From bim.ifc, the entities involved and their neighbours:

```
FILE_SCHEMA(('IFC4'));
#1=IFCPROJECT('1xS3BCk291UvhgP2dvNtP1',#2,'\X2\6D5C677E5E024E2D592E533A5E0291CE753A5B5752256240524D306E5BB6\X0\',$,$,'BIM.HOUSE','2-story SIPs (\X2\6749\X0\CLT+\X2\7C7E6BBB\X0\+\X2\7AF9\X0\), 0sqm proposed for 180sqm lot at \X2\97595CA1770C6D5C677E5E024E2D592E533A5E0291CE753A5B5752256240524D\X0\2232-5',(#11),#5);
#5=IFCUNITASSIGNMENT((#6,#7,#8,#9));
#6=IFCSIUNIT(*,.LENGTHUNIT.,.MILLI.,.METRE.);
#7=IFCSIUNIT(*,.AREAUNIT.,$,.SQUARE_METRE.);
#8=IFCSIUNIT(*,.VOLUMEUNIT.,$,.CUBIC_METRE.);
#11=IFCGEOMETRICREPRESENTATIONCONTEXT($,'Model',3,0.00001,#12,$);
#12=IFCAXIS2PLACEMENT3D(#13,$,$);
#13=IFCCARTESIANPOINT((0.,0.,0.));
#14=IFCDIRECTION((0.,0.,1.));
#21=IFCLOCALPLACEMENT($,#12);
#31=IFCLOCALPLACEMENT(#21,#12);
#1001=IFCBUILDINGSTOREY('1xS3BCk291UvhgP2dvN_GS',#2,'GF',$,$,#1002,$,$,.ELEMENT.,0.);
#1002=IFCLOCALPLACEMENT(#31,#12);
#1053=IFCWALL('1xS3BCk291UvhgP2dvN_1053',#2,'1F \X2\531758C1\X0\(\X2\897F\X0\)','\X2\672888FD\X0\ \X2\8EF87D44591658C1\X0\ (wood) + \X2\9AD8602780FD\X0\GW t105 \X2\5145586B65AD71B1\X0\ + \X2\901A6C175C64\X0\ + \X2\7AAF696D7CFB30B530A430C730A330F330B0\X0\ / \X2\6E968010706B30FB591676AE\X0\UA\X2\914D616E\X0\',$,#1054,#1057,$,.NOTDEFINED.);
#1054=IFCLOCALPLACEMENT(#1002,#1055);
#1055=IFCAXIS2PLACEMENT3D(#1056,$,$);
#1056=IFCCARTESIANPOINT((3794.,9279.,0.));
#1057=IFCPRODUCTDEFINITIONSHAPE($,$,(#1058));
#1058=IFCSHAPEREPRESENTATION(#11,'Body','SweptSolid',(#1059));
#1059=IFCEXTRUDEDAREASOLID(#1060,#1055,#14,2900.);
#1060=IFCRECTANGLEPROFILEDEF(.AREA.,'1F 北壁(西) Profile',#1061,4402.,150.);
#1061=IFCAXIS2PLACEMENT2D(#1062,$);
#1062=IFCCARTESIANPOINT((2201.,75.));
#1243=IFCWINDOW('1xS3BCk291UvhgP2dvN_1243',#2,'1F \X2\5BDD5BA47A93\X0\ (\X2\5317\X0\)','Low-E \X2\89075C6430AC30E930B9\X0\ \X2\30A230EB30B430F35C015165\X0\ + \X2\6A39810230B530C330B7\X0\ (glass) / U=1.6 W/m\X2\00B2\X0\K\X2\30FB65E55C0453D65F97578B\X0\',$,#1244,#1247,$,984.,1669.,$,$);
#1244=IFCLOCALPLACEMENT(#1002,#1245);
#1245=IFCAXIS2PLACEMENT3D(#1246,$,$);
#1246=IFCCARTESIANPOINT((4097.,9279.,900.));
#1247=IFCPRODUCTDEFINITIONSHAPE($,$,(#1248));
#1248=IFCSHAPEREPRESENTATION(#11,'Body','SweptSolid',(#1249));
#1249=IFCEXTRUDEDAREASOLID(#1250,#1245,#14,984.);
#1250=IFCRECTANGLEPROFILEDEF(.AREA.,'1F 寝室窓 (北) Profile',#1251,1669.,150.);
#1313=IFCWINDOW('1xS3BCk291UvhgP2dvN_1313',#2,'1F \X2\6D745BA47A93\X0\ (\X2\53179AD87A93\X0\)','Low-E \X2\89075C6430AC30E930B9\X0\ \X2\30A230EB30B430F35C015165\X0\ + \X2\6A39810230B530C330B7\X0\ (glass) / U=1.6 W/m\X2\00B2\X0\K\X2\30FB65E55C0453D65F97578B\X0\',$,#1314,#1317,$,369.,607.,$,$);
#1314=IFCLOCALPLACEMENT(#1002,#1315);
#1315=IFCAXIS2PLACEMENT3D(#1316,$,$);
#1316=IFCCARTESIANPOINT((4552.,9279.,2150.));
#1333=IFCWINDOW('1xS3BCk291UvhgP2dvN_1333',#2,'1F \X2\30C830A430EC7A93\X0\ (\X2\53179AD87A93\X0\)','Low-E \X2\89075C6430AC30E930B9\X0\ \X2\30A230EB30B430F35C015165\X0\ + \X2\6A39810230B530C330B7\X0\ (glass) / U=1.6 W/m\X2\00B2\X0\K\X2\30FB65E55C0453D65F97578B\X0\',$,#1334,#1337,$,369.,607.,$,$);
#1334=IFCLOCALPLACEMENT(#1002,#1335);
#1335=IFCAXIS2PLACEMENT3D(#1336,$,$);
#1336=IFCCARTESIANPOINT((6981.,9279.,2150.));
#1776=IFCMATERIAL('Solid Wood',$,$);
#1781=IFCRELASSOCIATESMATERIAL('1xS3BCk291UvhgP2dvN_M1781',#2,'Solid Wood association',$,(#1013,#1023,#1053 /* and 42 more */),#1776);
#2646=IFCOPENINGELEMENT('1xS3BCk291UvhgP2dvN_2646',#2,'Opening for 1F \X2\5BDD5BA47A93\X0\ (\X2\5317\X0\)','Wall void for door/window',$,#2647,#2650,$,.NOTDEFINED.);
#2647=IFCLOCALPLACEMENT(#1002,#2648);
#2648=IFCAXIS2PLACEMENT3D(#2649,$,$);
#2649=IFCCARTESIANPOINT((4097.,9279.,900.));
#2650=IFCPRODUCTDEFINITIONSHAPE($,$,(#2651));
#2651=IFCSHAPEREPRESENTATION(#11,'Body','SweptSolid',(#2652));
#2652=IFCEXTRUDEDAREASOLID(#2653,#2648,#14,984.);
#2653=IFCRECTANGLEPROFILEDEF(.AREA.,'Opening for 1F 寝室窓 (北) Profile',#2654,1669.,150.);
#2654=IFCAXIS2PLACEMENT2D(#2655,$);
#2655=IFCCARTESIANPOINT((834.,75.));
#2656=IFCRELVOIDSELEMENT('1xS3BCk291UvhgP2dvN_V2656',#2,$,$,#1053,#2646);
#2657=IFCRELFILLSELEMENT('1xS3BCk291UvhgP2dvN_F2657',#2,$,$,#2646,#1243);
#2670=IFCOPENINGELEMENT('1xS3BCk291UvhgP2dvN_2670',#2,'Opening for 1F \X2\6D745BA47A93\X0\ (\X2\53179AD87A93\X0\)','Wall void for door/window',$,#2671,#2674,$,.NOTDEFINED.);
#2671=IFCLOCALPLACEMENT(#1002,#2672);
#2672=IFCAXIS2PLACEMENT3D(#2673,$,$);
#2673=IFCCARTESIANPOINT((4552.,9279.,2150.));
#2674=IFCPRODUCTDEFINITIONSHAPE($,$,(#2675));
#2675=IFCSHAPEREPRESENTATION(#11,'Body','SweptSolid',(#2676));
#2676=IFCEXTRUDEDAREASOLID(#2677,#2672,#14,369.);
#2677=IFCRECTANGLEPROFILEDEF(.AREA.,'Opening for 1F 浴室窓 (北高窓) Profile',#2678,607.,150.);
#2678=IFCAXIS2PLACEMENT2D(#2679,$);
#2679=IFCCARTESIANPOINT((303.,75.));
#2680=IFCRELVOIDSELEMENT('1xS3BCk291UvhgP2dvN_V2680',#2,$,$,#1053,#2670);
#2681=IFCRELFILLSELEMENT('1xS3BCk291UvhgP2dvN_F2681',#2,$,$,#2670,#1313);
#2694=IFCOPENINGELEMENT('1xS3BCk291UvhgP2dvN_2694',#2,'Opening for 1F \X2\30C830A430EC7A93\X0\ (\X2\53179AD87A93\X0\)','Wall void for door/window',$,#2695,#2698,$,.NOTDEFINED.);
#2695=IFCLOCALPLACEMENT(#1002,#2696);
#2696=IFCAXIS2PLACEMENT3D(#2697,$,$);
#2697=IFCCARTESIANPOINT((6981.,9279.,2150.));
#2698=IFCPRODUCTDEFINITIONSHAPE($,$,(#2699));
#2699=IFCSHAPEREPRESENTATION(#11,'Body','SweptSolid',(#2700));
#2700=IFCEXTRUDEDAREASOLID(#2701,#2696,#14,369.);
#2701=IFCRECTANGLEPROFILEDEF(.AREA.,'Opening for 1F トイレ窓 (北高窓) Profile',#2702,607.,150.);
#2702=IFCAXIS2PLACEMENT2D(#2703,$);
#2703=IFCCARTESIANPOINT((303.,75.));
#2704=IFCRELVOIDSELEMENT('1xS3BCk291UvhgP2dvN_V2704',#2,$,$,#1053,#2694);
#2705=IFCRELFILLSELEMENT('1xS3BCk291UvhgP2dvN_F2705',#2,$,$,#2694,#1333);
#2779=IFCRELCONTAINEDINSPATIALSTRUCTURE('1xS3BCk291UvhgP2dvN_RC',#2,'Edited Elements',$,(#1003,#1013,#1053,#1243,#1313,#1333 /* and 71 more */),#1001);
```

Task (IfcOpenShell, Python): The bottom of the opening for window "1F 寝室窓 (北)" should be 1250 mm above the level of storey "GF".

```python
import numpy as np
import ifcopenshell
import ifcopenshell.api.geometry
import ifcopenshell.geom
import ifcopenshell.util.element
import ifcopenshell.util.placement
import ifcopenshell.util.shape
import ifcopenshell.util.unit

model = ifcopenshell.open("bim.ifc")
unit_scale = ifcopenshell.util.unit.calculate_unit_scale(model)

window = model.by_id(1243)
opening = window.FillsVoids[0].RelatingOpeningElement
storey = ifcopenshell.util.element.get_container(window, ifc_class="IfcBuildingStorey")
level = ifcopenshell.util.placement.get_local_placement(storey.ObjectPlacement)[2, 3]

# The opening's origin need not be at the sill, so measure its lowest point.
shape = ifcopenshell.geom.create_shape(ifcopenshell.geom.settings(), opening)
bottom = ifcopenshell.util.shape.get_shape_bottom_elevation(shape, shape.geometry) / unit_scale
dz = level + 1250.0 - bottom

shift = np.array([0.0, 0.0, dz])
# The window is not placed relative to its opening, so move both.
for product in (opening, window):
    matrix = ifcopenshell.util.placement.get_local_placement(product.ObjectPlacement)
    matrix[:3, 3] += shift
    ifcopenshell.api.geometry.edit_object_placement(model, product=product, matrix=matrix, is_si=False)

print(f"moved by {dz * unit_scale:+.3f} m")

model.write("bim_updated.ifc")
```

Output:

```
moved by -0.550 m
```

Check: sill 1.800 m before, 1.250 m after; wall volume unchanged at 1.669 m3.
